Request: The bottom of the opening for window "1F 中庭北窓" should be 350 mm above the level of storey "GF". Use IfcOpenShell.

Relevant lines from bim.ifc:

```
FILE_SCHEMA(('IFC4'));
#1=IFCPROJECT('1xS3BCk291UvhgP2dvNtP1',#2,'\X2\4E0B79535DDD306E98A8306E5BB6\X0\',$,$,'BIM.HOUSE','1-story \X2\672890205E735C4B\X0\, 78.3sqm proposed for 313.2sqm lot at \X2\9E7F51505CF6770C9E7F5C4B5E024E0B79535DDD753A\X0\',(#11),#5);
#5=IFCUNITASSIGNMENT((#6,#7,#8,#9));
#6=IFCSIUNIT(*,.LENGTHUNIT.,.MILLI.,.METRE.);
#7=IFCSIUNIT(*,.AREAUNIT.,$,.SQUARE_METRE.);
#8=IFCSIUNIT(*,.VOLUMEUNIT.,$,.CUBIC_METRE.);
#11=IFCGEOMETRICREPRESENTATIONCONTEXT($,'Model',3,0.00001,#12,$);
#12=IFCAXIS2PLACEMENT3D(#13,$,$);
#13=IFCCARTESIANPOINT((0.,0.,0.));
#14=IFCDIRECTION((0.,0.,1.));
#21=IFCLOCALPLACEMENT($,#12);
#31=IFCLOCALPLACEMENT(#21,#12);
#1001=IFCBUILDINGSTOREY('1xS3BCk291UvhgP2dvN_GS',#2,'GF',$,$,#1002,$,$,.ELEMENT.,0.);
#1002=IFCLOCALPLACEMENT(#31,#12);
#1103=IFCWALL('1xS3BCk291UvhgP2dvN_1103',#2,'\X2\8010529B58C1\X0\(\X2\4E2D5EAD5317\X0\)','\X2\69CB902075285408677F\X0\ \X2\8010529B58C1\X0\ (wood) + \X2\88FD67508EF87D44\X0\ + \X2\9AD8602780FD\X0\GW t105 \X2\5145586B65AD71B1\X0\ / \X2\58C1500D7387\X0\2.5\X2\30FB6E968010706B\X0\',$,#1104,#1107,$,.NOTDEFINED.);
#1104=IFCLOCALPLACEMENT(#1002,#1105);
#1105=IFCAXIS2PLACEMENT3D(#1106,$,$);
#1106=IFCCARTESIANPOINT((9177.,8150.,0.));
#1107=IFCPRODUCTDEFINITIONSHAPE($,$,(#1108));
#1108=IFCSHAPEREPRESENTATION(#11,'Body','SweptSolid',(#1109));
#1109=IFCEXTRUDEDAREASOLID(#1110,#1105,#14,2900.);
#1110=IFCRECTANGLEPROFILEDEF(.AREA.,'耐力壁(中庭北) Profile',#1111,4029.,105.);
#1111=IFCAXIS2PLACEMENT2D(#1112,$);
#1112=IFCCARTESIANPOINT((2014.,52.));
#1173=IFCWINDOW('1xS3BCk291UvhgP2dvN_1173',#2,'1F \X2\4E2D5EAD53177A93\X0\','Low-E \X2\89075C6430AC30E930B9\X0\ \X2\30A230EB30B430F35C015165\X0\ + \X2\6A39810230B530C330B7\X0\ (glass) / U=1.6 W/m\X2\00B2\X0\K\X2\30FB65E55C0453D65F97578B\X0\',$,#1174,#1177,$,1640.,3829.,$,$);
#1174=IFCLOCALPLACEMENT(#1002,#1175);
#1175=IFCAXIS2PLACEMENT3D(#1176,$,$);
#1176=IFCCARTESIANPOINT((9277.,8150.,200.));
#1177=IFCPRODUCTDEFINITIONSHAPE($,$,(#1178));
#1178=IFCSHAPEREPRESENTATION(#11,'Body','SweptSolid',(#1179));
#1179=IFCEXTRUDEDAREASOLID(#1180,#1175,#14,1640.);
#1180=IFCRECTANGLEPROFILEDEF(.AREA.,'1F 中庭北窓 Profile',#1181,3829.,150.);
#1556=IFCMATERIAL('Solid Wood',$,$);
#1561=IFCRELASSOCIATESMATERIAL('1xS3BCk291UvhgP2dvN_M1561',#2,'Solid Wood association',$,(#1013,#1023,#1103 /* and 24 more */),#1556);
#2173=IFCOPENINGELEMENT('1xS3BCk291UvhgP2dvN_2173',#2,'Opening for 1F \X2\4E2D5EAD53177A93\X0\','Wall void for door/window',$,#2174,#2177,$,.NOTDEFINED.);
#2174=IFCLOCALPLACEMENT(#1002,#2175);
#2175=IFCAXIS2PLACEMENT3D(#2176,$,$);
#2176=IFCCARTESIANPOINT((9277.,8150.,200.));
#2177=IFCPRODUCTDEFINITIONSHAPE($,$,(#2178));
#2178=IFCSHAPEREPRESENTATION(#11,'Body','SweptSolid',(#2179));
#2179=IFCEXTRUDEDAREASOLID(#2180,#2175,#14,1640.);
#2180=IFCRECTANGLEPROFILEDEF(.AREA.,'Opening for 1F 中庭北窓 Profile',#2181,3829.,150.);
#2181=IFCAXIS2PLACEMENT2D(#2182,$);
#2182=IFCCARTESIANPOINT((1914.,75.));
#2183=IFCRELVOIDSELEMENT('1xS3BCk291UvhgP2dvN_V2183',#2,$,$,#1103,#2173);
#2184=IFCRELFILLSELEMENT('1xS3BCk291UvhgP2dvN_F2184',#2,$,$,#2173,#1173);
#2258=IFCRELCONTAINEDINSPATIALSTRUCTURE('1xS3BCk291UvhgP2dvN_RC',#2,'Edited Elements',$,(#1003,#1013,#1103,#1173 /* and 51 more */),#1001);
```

```python
import numpy as np
import ifcopenshell
import ifcopenshell.api.geometry
import ifcopenshell.geom
import ifcopenshell.util.element
import ifcopenshell.util.placement
import ifcopenshell.util.shape
import ifcopenshell.util.unit

model = ifcopenshell.open("bim.ifc")
unit_scale = ifcopenshell.util.unit.calculate_unit_scale(model)

window = model.by_id(1173)
opening = window.FillsVoids[0].RelatingOpeningElement
storey = ifcopenshell.util.element.get_container(window, ifc_class="IfcBuildingStorey")
level = ifcopenshell.util.placement.get_local_placement(storey.ObjectPlacement)[2, 3]

# The opening's origin need not be at the sill, so measure its lowest point.
shape = ifcopenshell.geom.create_shape(ifcopenshell.geom.settings(), opening)
bottom = ifcopenshell.util.shape.get_shape_bottom_elevation(shape, shape.geometry) / unit_scale
dz = level + 0.35 / unit_scale - bottom

shift = np.array([0.0, 0.0, dz])
# The window is not placed relative to its opening, so move both.
for product in (opening, window):
    matrix = ifcopenshell.util.placement.get_local_placement(product.ObjectPlacement)
    matrix[:3, 3] += shift
    ifcopenshell.api.geometry.edit_object_placement(model, product=product, matrix=matrix, is_si=False)

print(f"moved by {dz * unit_scale:+.3f} m")

model.write("bim_v2.ifc")
```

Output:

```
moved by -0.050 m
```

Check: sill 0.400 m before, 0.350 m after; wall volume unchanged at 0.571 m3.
